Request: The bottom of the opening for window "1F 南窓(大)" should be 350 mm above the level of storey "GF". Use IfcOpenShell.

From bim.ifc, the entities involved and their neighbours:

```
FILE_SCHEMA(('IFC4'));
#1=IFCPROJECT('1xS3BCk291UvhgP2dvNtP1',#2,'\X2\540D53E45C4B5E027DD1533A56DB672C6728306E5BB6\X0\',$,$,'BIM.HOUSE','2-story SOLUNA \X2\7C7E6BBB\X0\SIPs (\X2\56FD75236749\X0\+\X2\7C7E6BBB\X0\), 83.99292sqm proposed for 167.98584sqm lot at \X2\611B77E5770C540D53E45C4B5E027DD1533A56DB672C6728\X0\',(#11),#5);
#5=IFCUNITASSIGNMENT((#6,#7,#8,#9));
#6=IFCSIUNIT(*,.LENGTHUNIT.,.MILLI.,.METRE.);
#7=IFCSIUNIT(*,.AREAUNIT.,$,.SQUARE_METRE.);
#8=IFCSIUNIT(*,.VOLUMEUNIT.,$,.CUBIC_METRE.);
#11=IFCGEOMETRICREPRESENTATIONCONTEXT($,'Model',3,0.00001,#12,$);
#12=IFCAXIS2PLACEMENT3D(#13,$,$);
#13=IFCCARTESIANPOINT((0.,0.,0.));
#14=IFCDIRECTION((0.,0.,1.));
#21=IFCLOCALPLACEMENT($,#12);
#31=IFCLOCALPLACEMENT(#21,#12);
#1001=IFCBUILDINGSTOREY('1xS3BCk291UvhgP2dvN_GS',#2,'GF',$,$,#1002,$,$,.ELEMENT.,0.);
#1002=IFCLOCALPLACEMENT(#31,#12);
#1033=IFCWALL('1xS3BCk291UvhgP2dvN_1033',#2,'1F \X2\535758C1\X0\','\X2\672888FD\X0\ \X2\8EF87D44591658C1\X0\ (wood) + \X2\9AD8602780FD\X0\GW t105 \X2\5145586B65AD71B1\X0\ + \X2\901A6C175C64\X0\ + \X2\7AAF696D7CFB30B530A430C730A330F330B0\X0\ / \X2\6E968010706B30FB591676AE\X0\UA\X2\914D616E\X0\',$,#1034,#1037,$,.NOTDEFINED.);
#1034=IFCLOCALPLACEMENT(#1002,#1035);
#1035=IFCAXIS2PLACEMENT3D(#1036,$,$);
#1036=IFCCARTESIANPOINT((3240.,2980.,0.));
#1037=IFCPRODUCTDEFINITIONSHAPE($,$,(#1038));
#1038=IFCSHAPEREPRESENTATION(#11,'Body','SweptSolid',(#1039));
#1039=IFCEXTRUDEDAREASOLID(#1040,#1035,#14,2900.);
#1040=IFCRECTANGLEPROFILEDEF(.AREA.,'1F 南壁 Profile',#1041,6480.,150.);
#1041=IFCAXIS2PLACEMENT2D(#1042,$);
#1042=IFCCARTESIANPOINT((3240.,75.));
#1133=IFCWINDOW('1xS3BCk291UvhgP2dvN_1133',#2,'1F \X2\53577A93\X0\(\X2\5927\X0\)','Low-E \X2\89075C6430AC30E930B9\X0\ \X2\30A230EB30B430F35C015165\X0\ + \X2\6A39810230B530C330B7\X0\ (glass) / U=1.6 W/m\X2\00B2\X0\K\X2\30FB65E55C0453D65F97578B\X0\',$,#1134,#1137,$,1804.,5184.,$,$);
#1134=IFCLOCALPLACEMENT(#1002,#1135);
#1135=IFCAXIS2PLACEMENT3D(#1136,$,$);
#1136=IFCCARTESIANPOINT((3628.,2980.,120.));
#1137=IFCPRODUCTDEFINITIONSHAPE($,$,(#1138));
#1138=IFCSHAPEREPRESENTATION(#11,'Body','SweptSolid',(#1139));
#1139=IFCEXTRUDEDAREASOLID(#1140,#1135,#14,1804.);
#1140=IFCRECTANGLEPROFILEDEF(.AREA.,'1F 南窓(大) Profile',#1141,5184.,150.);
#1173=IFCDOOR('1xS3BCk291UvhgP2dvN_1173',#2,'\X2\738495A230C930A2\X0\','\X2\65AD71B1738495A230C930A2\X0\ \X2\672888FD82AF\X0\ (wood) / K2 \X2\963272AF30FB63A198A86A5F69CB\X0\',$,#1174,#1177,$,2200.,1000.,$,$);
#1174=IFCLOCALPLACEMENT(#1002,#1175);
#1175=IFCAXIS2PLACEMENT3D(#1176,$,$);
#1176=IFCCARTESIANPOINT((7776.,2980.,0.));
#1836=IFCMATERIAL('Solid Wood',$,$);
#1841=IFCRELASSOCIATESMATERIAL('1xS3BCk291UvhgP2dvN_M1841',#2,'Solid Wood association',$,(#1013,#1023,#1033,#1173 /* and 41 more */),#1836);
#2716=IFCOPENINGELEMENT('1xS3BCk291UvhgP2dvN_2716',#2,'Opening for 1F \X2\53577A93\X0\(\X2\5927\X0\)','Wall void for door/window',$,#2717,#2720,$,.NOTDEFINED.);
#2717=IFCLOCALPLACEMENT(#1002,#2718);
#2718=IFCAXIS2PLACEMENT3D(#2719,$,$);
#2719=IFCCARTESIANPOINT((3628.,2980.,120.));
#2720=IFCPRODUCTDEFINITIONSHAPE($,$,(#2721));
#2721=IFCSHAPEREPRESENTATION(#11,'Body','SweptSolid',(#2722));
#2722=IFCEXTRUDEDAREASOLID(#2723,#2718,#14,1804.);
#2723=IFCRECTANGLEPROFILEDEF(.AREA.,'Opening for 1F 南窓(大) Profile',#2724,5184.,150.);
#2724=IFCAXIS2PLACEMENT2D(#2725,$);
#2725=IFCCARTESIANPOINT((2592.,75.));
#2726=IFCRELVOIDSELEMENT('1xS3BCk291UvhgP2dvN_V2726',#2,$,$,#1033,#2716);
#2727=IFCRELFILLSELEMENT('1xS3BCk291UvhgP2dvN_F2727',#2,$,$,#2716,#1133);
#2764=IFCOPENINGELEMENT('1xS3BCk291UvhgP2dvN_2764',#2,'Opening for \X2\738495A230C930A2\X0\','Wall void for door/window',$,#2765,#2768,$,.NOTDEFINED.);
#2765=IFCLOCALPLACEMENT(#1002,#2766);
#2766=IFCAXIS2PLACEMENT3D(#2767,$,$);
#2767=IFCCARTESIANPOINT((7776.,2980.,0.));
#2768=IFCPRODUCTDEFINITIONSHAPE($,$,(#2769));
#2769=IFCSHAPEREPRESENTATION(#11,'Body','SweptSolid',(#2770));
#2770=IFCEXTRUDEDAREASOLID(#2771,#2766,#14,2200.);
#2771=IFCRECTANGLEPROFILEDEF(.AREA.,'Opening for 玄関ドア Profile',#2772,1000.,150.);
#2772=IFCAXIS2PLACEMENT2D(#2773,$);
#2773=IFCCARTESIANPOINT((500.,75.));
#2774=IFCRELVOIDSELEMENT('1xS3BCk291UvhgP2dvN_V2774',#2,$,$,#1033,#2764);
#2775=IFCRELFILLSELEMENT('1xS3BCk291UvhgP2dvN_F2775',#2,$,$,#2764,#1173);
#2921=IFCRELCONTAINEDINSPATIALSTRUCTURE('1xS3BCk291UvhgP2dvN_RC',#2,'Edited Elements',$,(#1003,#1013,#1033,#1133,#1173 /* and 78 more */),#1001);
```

```python
import numpy as np
import ifcopenshell
import ifcopenshell.api.geometry
import ifcopenshell.geom
import ifcopenshell.util.element
import ifcopenshell.util.placement
import ifcopenshell.util.shape
import ifcopenshell.util.unit

model = ifcopenshell.open("bim.ifc")
unit_scale = ifcopenshell.util.unit.calculate_unit_scale(model)

window = model.by_guid("1xS3BCk291UvhgP2dvN_1133")
opening = window.FillsVoids[0].RelatingOpeningElement
storey = ifcopenshell.util.element.get_container(window, ifc_class="IfcBuildingStorey")
level = ifcopenshell.util.placement.get_local_placement(storey.ObjectPlacement)[2, 3]

# The opening's origin need not be at the sill, so measure its lowest point.
shape = ifcopenshell.geom.create_shape(ifcopenshell.geom.settings(), opening)
bottom = ifcopenshell.util.shape.get_shape_bottom_elevation(shape, shape.geometry) / unit_scale
dz = level + 0.35 / unit_scale - bottom

shift = np.array([0.0, 0.0, dz])
# The window is not placed relative to its opening, so move both.
for product in (opening, window):
    matrix = ifcopenshell.util.placement.get_local_placement(product.ObjectPlacement)
    matrix[:3, 3] += shift
    ifcopenshell.api.geometry.edit_object_placement(model, product=product, matrix=matrix, is_si=False)

print(f"moved by {dz * unit_scale:+.3f} m")

model.write("bim_edited.ifc")
```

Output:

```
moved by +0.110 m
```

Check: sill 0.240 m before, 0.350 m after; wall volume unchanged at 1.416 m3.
